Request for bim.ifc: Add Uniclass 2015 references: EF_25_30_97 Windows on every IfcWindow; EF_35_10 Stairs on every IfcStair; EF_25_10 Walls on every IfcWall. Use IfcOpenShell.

First a look at what the model holds.

```python
import ifcopenshell

model = ifcopenshell.open("bim.ifc")
print(model.schema)
print("classifications:", [c.Name for c in model.by_type("IfcClassification")])
for ifc_class in ("IfcDoor", "IfcRoof", "IfcStair", "IfcWall", "IfcWindow"):
    print(ifc_class, len(model.by_type(ifc_class)))
```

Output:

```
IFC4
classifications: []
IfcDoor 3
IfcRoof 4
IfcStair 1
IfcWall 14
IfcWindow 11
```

```python
import ifcopenshell
import ifcopenshell.api.classification

model = ifcopenshell.open("bim.ifc")

system = ifcopenshell.api.classification.add_classification(model, classification="Uniclass 2015")

codes = {
    "IfcWindow": ("EF_25_30_97", "Windows"),
    "IfcStair": ("EF_35_10", "Stairs"),
    "IfcWall": ("EF_25_10", "Walls"),
}
for ifc_class, (code, name) in codes.items():
    products = model.by_type(ifc_class)
    ifcopenshell.api.classification.add_reference(
        model, products=products, classification=system, identification=code, name=name
    )
    print(code, len(products))

model.write("bim-out.ifc")
```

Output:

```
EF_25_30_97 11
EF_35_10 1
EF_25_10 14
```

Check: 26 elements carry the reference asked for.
